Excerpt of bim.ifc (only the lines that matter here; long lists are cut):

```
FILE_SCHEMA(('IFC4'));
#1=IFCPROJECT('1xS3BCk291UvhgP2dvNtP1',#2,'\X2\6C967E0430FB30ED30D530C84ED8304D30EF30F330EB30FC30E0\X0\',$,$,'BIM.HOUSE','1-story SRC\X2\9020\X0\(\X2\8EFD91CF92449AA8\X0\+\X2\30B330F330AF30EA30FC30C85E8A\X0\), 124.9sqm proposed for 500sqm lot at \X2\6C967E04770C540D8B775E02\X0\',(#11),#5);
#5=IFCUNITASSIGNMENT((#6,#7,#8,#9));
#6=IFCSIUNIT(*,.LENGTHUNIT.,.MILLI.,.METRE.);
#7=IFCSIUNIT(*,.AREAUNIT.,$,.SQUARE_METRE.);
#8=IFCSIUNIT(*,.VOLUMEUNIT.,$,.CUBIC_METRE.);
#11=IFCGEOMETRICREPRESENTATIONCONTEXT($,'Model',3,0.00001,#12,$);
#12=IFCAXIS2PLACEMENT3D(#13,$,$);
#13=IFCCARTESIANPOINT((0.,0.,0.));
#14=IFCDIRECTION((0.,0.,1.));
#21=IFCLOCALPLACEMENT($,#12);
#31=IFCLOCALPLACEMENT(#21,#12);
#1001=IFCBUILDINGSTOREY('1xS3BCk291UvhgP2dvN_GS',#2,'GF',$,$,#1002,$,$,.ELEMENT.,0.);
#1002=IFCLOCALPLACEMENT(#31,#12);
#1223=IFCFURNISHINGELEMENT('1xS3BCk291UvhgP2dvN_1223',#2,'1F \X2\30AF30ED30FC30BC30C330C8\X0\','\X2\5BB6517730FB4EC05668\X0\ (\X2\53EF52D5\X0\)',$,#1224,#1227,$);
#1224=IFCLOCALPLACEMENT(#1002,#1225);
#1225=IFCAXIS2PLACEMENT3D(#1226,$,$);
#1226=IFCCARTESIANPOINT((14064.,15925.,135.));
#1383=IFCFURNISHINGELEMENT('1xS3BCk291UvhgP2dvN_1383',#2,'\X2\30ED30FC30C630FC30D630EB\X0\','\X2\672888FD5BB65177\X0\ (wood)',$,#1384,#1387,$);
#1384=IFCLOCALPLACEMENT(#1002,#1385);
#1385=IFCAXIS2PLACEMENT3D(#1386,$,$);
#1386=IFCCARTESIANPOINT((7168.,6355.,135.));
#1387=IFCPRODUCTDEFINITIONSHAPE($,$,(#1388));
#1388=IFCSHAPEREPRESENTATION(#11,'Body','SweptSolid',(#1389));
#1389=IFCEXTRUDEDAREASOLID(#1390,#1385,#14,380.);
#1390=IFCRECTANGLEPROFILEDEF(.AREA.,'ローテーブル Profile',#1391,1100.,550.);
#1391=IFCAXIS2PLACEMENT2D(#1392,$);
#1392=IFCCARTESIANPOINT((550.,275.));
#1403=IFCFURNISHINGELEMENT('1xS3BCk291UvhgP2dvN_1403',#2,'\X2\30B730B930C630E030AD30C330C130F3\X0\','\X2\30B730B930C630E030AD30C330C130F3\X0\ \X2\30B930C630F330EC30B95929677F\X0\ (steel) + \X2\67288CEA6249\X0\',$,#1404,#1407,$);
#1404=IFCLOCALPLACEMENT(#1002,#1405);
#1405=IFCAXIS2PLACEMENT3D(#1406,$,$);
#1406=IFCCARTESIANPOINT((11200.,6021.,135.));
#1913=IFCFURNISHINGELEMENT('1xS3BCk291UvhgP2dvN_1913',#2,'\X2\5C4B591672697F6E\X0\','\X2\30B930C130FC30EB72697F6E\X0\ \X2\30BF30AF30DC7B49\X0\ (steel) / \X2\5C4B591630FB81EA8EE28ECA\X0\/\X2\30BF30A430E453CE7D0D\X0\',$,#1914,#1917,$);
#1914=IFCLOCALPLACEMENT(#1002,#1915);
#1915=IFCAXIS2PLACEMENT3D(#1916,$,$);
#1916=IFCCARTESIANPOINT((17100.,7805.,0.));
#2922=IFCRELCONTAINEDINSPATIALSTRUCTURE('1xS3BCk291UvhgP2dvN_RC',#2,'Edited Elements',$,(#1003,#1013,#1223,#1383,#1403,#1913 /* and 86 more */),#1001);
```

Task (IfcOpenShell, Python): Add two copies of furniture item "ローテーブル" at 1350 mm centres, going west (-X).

```python
import numpy as np
import ifcopenshell
import ifcopenshell.api.geometry
import ifcopenshell.api.root
import ifcopenshell.util.element
import ifcopenshell.util.placement

model = ifcopenshell.open("bim.ifc")


def reuse_history(source, copy):
    """copy_class also copies each property set's owner history, people and application; keep the originals."""
    for rel in copy.IsDefinedBy:
        if rel.is_a("IfcRelDefinesByProperties") and (history := rel.RelatingPropertyDefinition.OwnerHistory):
            rel.RelatingPropertyDefinition.OwnerHistory = source.OwnerHistory
            ifcopenshell.util.element.remove_deep2(model, history)


source = model.by_guid("1xS3BCk291UvhgP2dvN_1383")
base = ifcopenshell.util.placement.get_local_placement(source.ObjectPlacement)
step = np.array([-1.0, 0.0, 0.0]) * 1350.0

for i in range(1, 3):
    copy = ifcopenshell.api.root.copy_class(model, product=source)
    copy.Representation = ifcopenshell.util.element.copy_deep(
        model, source.Representation, exclude=["IfcGeometricRepresentationContext", "IfcRepresentationMap"]
    )
    reuse_history(source, copy)
    matrix = base.copy()
    matrix[:3, 3] += i * step
    print("added at", matrix[:3, 3].round(3) + 0.0)
    ifcopenshell.api.geometry.edit_object_placement(model, product=copy, matrix=matrix, is_si=False)

model.write("bim-out.ifc")
```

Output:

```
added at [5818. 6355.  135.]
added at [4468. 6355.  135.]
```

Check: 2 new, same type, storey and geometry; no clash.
